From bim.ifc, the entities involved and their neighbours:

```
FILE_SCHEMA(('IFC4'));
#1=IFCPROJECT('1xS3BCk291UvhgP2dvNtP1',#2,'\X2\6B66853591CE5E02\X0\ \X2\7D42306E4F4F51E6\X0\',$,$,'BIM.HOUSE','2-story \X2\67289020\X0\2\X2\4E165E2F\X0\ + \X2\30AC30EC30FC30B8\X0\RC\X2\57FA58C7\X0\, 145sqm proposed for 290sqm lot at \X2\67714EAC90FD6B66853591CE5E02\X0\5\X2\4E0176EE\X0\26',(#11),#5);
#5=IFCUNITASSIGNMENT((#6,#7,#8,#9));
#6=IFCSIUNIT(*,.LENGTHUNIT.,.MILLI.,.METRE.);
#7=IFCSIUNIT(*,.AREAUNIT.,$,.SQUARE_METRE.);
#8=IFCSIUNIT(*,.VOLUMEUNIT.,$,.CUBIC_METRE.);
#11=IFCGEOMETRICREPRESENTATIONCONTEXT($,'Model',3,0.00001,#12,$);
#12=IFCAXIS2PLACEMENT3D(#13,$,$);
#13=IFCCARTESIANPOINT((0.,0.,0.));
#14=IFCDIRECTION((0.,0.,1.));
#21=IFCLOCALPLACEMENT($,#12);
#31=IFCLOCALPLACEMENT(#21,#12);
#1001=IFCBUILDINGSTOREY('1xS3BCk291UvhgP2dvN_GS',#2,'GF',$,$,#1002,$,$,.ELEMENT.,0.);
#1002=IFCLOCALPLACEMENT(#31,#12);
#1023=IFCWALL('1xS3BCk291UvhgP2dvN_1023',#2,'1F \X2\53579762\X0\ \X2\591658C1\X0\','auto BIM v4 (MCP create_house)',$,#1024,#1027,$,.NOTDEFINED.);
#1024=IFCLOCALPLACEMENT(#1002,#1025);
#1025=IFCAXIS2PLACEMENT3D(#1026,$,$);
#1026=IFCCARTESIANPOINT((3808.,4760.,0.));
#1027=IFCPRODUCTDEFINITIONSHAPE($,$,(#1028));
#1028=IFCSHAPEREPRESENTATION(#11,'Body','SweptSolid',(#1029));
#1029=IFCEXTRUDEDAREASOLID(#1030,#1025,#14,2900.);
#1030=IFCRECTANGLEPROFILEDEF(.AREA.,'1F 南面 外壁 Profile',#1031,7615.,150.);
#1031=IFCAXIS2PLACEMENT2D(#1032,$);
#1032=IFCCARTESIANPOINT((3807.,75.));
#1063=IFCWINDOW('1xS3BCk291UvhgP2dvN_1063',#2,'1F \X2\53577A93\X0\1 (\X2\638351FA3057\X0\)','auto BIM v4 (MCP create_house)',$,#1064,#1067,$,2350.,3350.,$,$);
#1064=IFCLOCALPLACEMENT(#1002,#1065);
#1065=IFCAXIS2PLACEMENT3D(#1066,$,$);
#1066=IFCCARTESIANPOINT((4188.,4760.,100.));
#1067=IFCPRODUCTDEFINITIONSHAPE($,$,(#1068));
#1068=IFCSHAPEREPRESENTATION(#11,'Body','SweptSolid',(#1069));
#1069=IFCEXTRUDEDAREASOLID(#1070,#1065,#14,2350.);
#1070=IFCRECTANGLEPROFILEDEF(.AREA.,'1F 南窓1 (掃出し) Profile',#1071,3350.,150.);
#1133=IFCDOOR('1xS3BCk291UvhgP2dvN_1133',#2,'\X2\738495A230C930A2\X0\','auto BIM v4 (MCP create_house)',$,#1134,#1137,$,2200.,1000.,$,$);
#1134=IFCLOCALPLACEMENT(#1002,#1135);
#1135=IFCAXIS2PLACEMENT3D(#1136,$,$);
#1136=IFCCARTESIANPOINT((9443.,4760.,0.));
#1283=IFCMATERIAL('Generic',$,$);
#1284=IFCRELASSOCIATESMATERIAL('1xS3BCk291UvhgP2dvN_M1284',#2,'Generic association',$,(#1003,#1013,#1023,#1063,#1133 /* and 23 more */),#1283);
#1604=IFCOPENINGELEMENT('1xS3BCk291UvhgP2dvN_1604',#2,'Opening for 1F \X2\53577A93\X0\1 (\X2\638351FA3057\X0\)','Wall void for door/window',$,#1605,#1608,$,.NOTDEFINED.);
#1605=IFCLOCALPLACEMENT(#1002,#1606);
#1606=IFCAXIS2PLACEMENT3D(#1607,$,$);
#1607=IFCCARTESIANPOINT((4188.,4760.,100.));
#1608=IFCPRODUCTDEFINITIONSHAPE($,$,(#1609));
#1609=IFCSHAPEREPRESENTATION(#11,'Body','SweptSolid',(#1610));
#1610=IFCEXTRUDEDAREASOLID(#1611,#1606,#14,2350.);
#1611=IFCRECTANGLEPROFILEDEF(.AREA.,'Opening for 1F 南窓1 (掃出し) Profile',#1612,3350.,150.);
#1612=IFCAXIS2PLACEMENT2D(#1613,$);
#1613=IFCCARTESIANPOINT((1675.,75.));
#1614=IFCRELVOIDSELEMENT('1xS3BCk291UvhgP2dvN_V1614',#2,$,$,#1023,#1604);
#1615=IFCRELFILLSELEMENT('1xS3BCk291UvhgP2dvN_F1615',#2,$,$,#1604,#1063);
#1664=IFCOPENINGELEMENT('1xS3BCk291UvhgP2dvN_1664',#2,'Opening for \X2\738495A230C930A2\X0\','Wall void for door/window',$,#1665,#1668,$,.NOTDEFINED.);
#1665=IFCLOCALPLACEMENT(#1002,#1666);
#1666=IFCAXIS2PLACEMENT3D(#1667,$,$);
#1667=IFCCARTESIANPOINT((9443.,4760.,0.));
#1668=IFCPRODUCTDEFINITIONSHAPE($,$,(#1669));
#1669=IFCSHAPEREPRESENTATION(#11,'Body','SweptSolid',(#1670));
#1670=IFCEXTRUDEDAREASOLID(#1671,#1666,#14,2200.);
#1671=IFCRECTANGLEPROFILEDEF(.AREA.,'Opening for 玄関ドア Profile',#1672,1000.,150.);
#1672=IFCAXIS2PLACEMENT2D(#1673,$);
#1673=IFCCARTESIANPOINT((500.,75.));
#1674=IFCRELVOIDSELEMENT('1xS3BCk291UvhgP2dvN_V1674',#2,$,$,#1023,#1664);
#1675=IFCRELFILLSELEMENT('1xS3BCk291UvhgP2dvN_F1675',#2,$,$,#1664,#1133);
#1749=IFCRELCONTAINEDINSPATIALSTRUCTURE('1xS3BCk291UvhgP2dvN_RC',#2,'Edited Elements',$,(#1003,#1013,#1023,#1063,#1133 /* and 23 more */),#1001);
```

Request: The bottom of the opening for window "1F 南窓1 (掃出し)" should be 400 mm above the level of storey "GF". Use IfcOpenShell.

```python
import numpy as np
import ifcopenshell
import ifcopenshell.api.geometry
import ifcopenshell.geom
import ifcopenshell.util.element
import ifcopenshell.util.placement
import ifcopenshell.util.shape
import ifcopenshell.util.unit

model = ifcopenshell.open("bim.ifc")
unit_scale = ifcopenshell.util.unit.calculate_unit_scale(model)

window = model.by_guid("1xS3BCk291UvhgP2dvN_1063")
opening = window.FillsVoids[0].RelatingOpeningElement
storey = ifcopenshell.util.element.get_container(window, ifc_class="IfcBuildingStorey")
level = ifcopenshell.util.placement.get_local_placement(storey.ObjectPlacement)[2, 3]

# The opening's origin need not be at the sill, so measure its lowest point.
shape = ifcopenshell.geom.create_shape(ifcopenshell.geom.settings(), opening)
bottom = ifcopenshell.util.shape.get_shape_bottom_elevation(shape, shape.geometry) / unit_scale
dz = level + 400.0 - bottom

shift = np.array([0.0, 0.0, dz])
# The window is not placed relative to its opening, so move both.
for product in (opening, window):
    matrix = ifcopenshell.util.placement.get_local_placement(product.ObjectPlacement)
    matrix[:3, 3] += shift
    ifcopenshell.api.geometry.edit_object_placement(model, product=product, matrix=matrix, is_si=False)

print(f"moved by {dz * unit_scale:+.3f} m")

model.write("bim-out.ifc")
```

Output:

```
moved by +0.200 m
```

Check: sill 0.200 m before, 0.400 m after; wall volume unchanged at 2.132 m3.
